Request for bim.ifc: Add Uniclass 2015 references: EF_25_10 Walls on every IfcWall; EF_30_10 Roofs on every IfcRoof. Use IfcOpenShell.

First a look at what the model holds.

```python
import ifcopenshell

model = ifcopenshell.open("bim.ifc")
print(model.schema)
print("classifications:", [c.Name for c in model.by_type("IfcClassification")])
for ifc_class in ("IfcDoor", "IfcRoof", "IfcStair", "IfcWall", "IfcWindow"):
    print(ifc_class, len(model.by_type(ifc_class)))
```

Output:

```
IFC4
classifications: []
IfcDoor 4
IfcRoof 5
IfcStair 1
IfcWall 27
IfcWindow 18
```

```python
import ifcopenshell
import ifcopenshell.api.classification

model = ifcopenshell.open("bim.ifc")

system = ifcopenshell.api.classification.add_classification(model, classification="Uniclass 2015")

codes = {
    "IfcWall": ("EF_25_10", "Walls"),
    "IfcRoof": ("EF_30_10", "Roofs"),
}
for ifc_class, (code, name) in codes.items():
    products = model.by_type(ifc_class)
    ifcopenshell.api.classification.add_reference(
        model, products=products, classification=system, identification=code, name=name
    )
    print(code, len(products))

model.write("bim_v2.ifc")
```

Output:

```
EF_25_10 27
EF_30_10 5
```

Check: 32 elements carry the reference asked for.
